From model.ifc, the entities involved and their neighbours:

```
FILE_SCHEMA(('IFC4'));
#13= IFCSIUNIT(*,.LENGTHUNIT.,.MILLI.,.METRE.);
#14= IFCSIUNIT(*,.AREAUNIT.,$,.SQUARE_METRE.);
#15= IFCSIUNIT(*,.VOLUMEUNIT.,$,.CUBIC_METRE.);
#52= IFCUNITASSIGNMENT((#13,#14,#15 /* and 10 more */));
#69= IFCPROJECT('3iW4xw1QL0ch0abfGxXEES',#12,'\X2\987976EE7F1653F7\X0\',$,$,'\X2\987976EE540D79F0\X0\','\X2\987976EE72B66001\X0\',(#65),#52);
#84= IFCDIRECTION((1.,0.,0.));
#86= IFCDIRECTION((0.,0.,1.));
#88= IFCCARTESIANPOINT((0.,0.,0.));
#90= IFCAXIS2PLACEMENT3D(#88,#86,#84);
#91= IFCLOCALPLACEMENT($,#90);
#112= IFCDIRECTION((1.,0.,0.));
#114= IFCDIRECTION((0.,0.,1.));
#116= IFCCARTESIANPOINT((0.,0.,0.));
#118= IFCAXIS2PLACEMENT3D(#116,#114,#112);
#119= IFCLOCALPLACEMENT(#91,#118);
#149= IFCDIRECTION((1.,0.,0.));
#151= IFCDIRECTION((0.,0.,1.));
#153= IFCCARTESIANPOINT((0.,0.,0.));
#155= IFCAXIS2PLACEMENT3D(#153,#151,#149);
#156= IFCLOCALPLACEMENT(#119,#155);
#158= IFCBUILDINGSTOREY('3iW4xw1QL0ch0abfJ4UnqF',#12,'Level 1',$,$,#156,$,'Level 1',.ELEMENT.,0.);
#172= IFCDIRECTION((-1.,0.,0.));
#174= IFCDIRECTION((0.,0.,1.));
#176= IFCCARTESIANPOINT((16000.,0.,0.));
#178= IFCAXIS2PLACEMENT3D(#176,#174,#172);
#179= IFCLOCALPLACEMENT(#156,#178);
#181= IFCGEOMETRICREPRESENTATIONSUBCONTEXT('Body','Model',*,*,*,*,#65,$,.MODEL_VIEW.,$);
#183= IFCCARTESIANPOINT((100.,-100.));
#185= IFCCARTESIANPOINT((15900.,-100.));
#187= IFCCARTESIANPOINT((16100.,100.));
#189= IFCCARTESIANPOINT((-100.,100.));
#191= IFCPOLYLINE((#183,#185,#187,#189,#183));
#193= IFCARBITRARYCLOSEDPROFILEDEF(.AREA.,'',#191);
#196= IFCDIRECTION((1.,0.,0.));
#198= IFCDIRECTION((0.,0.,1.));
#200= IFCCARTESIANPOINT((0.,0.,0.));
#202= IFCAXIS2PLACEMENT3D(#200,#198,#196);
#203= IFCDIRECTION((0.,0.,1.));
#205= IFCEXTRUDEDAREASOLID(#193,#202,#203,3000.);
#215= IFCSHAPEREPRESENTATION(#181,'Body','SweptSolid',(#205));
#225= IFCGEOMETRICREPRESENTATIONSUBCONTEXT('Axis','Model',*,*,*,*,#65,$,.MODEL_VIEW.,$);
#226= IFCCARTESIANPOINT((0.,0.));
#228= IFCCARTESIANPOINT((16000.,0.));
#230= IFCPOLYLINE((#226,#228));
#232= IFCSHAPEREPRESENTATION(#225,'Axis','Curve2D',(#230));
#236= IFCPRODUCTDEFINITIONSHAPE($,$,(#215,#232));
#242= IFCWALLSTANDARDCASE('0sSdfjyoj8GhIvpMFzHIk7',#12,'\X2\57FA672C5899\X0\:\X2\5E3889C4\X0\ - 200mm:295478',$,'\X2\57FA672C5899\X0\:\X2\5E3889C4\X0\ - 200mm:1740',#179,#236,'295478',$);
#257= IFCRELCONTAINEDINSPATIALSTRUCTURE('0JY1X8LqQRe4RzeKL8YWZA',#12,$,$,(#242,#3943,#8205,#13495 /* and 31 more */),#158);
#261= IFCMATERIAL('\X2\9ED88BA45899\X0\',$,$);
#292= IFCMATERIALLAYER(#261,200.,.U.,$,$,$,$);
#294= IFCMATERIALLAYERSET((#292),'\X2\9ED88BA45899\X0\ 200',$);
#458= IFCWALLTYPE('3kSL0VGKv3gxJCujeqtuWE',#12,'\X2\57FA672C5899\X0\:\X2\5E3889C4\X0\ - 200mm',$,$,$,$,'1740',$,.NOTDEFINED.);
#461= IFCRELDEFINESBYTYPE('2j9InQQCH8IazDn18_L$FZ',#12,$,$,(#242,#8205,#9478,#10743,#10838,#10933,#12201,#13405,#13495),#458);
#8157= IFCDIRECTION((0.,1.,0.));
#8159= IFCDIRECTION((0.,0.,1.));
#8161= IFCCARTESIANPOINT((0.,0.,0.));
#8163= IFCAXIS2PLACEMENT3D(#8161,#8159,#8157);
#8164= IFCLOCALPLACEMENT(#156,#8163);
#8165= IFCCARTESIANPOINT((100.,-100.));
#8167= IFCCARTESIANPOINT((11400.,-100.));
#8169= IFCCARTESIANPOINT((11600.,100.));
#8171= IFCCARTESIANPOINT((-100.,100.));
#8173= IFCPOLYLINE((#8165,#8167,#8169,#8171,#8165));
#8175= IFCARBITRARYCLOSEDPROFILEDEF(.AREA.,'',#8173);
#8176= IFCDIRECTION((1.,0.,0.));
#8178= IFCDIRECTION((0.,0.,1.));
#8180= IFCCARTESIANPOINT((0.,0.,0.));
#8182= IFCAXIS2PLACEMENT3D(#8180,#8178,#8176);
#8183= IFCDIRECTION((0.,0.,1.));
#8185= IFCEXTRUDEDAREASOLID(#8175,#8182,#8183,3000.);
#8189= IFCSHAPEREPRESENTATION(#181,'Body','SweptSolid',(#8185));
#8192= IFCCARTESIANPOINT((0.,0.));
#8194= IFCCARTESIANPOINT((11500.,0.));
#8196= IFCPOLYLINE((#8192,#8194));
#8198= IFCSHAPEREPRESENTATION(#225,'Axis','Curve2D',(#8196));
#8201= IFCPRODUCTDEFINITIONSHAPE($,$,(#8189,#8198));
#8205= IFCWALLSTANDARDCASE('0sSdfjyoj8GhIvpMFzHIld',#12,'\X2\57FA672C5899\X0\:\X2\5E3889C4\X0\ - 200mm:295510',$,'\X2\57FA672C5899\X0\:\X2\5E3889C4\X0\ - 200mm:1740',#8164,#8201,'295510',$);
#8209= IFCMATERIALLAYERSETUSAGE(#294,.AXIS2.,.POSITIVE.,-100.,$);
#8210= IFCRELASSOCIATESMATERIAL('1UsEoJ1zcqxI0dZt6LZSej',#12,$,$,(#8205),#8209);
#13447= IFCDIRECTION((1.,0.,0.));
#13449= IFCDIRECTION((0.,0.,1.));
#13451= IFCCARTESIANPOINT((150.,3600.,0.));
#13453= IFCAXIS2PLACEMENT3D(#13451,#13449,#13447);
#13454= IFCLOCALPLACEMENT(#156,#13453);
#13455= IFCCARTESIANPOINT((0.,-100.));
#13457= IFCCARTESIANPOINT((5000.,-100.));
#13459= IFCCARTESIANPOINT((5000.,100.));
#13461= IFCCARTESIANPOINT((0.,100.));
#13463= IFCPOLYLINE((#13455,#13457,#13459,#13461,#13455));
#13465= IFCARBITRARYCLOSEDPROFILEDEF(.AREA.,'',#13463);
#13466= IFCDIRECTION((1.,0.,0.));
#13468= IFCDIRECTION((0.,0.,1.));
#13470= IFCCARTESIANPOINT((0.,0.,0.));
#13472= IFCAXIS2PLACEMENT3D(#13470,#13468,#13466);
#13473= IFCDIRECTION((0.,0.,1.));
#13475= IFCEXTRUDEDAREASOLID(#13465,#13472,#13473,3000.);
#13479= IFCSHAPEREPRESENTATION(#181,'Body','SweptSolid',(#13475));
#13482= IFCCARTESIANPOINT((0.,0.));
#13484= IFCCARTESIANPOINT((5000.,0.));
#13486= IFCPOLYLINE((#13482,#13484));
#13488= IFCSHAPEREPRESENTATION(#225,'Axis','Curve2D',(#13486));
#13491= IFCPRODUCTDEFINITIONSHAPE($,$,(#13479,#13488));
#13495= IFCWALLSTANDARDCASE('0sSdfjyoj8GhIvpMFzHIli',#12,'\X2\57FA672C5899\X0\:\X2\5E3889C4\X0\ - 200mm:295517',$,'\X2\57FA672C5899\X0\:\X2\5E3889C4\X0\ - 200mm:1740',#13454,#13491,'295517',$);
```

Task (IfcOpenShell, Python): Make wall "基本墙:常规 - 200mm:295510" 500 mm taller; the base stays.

```python
import ifcopenshell
import ifcopenshell.geom
import ifcopenshell.util.representation
import ifcopenshell.util.shape
import ifcopenshell.util.unit

model = ifcopenshell.open("model.ifc")
unit_scale = ifcopenshell.util.unit.calculate_unit_scale(model)
settings = ifcopenshell.geom.settings()


def volume(element):
    """Net volume in cubic metres, openings subtracted."""
    shape = ifcopenshell.geom.create_shape(settings, element)
    return ifcopenshell.util.shape.get_volume(shape.geometry)


wall = model.by_id(8205)
before = volume(wall)

body = ifcopenshell.util.representation.get_representation(wall, "Model", "Body")
solid = body.Items[0]
old_height = solid.Depth
solid.Depth += 0.5 / unit_scale
after = volume(wall)

print(f"height {old_height:g} -> {solid.Depth:g}, volume {before:.3f} -> {after:.3f} m3")

model.write("model-out.ifc")
```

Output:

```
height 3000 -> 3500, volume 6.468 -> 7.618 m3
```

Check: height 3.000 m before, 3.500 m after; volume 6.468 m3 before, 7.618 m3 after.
